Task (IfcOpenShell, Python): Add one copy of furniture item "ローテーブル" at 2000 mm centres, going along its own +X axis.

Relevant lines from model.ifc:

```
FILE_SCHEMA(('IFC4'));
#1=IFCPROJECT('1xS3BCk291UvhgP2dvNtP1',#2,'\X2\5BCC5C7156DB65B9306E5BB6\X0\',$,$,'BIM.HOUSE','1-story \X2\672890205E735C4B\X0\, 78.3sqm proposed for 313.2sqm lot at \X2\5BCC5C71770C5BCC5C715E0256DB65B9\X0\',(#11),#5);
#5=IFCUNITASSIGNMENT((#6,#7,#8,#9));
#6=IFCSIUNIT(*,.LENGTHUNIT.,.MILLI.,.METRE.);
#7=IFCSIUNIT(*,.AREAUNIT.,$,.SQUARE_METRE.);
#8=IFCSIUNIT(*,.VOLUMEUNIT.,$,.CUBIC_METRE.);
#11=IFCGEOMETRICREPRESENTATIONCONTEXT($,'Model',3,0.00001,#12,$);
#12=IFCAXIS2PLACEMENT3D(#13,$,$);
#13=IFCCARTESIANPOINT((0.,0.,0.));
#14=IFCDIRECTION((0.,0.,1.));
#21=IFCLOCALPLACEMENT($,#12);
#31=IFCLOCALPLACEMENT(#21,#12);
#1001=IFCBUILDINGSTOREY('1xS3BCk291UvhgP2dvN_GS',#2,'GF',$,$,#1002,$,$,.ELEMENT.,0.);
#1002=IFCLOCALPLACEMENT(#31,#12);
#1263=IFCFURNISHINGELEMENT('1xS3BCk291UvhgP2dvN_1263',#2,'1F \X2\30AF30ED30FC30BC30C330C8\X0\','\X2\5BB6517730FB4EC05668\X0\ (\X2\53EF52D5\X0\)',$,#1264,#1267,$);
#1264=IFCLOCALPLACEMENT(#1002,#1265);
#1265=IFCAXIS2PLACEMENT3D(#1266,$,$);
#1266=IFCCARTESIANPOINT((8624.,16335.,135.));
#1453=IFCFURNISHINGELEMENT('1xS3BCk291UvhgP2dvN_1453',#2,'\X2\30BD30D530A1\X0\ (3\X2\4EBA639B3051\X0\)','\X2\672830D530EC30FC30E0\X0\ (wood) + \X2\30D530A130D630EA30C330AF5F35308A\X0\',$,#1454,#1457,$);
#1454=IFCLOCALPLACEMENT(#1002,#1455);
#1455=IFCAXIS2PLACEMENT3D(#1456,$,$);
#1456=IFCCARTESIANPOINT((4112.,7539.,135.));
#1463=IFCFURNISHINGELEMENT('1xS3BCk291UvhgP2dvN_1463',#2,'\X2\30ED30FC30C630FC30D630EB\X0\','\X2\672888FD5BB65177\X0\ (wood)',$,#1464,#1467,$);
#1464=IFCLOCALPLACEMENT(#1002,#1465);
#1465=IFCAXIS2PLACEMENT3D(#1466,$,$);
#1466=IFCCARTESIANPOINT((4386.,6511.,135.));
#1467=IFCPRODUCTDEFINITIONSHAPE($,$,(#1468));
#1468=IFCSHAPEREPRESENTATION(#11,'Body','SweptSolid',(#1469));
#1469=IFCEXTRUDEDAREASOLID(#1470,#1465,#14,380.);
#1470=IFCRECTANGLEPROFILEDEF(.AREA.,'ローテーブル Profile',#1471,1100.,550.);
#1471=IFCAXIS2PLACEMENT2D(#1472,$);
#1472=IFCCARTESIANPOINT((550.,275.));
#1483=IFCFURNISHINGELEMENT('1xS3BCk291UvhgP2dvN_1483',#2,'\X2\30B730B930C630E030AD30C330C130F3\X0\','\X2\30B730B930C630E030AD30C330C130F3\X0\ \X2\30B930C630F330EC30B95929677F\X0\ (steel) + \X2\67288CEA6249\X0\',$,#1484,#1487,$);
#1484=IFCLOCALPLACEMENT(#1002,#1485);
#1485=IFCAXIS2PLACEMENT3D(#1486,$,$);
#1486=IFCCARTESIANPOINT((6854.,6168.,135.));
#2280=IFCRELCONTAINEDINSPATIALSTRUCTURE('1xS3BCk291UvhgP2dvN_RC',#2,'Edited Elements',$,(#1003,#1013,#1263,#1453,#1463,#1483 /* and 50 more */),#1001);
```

```python
import ifcopenshell
import ifcopenshell.api.geometry
import ifcopenshell.api.root
import ifcopenshell.util.element
import ifcopenshell.util.placement

model = ifcopenshell.open("model.ifc")


def reuse_history(source, copy):
    """copy_class also copies each property set's owner history, people and application; keep the originals."""
    for rel in copy.IsDefinedBy:
        if rel.is_a("IfcRelDefinesByProperties") and (history := rel.RelatingPropertyDefinition.OwnerHistory):
            rel.RelatingPropertyDefinition.OwnerHistory = source.OwnerHistory
            ifcopenshell.util.element.remove_deep2(model, history)


source = model.by_id(1463)
base = ifcopenshell.util.placement.get_local_placement(source.ObjectPlacement)
step = base[:3, 0] * 2000.0

for i in range(1, 2):
    copy = ifcopenshell.api.root.copy_class(model, product=source)
    copy.Representation = ifcopenshell.util.element.copy_deep(
        model, source.Representation, exclude=["IfcGeometricRepresentationContext", "IfcRepresentationMap"]
    )
    reuse_history(source, copy)
    matrix = base.copy()
    matrix[:3, 3] += i * step
    print("added at", matrix[:3, 3].round(3) + 0.0)
    ifcopenshell.api.geometry.edit_object_placement(model, product=copy, matrix=matrix, is_si=False)

model.write("model_edited.ifc")
```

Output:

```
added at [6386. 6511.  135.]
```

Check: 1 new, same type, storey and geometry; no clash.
